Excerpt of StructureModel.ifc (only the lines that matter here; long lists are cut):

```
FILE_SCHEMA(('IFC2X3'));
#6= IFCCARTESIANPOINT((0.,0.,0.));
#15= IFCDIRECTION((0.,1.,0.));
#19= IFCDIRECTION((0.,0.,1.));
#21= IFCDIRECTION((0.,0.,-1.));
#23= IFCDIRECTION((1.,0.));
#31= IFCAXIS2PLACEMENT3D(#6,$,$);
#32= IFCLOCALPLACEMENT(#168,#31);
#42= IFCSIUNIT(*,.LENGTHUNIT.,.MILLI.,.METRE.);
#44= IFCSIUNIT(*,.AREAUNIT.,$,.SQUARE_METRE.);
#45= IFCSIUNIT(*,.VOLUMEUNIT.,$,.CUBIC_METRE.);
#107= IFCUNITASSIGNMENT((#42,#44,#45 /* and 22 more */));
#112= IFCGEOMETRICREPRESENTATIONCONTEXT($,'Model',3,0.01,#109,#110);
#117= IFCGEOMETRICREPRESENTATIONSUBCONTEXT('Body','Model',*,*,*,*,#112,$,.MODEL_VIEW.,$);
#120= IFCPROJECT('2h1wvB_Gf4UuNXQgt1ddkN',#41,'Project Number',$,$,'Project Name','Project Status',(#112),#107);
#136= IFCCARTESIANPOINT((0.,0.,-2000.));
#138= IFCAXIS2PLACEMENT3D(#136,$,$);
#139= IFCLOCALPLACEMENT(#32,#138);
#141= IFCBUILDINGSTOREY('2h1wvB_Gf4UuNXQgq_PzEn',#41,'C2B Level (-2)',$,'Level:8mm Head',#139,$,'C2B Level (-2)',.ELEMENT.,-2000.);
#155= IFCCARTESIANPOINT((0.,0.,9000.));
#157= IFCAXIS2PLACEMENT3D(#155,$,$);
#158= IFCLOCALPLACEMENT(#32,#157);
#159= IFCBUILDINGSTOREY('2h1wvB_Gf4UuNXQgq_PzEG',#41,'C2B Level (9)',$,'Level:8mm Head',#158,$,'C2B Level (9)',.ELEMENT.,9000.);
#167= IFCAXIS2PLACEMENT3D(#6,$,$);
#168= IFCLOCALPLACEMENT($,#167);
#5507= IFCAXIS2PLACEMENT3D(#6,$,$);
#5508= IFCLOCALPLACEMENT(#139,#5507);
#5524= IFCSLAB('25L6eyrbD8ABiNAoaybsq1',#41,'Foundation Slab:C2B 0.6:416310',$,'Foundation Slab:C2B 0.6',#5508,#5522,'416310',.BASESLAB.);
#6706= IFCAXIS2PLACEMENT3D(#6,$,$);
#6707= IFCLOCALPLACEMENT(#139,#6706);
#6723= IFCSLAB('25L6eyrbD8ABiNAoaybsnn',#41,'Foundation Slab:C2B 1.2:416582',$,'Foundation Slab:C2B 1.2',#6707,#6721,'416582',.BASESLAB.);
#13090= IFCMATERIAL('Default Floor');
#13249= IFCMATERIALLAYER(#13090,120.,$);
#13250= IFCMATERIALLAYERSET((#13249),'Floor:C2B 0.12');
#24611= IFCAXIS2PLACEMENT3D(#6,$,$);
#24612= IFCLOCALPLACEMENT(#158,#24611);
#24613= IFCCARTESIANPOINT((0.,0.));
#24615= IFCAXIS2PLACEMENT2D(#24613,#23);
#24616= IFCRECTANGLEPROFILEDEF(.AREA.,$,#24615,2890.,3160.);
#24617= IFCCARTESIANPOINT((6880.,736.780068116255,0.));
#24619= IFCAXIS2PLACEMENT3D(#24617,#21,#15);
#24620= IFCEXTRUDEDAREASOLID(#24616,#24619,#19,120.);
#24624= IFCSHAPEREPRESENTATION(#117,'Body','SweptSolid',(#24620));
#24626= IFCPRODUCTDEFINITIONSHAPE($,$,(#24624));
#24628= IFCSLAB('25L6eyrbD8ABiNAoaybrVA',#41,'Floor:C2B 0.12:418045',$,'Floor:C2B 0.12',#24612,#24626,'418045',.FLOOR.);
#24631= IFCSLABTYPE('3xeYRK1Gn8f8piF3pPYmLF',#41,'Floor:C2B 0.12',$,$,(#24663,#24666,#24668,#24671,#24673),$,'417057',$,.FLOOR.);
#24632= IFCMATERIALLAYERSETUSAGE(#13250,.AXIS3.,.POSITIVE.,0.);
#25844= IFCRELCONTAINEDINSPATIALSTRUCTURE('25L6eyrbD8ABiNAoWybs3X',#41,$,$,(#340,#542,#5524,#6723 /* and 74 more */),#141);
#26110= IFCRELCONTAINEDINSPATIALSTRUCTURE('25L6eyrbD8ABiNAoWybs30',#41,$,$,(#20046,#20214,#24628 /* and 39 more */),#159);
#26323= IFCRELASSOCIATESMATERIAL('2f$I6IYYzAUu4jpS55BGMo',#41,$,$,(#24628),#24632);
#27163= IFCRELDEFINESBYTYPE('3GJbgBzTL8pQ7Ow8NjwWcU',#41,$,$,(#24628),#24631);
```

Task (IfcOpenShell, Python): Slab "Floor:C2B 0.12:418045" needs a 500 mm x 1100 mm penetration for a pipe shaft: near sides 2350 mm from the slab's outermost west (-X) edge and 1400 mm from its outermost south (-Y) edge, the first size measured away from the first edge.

```python
import numpy as np
import ifcopenshell
import ifcopenshell.api.feature
import ifcopenshell.api.geometry
import ifcopenshell.api.root
import ifcopenshell.geom
import ifcopenshell.util.placement
import ifcopenshell.util.representation
import ifcopenshell.util.shape
import ifcopenshell.util.unit

model = ifcopenshell.open("StructureModel.ifc")
unit_scale = ifcopenshell.util.unit.calculate_unit_scale(model)
settings = ifcopenshell.geom.settings()


def volume(element):
    """Net volume in cubic metres, openings subtracted."""
    shape = ifcopenshell.geom.create_shape(settings, element)
    return ifcopenshell.util.shape.get_volume(shape.geometry)


slab = model.by_id(24628)
before = volume(slab)

# Extent in the slab's own axes, in metres. The edges named are its -X and -Y sides.
slab_shape = ifcopenshell.geom.create_shape(settings, slab)
vertices = ifcopenshell.util.shape.get_vertices(slab_shape.geometry)
x_min, y_min, bottom = vertices.min(axis=0)
top = vertices[:, 2].max()

opening = ifcopenshell.api.root.create_entity(model, ifc_class="IfcOpeningElement", name="Pipe shaft opening")
context = ifcopenshell.util.representation.get_context(model, "Model", "Body", "MODEL_VIEW")
width, depth = 0.5, 1.1
outline = [(0.0, 0.0), (width, 0.0), (width, depth), (0.0, depth), (0.0, 0.0)]
# Overshoot both faces by 50 mm so the cut is clean.
shape = ifcopenshell.api.geometry.add_slab_representation(
    model, context=context, depth=top - bottom + 0.1, polyline=outline
)
ifcopenshell.api.geometry.assign_representation(model, product=opening, representation=shape)

matrix = ifcopenshell.util.placement.get_local_placement(slab.ObjectPlacement)
matrix[:, 3] = matrix @ np.append(np.array([x_min + 2.35, y_min + 1.4, bottom - 0.05]) / unit_scale, 1.0)
ifcopenshell.api.geometry.edit_object_placement(model, product=opening, matrix=matrix, is_si=False)
ifcopenshell.api.feature.add_feature(model, feature=opening, element=slab)

after = volume(slab)

print(f"slab volume {before:.3f} -> {after:.3f} m3")

model.write("StructureModel_edited.ifc")
```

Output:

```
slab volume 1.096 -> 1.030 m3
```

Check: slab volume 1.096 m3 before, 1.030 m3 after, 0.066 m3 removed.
